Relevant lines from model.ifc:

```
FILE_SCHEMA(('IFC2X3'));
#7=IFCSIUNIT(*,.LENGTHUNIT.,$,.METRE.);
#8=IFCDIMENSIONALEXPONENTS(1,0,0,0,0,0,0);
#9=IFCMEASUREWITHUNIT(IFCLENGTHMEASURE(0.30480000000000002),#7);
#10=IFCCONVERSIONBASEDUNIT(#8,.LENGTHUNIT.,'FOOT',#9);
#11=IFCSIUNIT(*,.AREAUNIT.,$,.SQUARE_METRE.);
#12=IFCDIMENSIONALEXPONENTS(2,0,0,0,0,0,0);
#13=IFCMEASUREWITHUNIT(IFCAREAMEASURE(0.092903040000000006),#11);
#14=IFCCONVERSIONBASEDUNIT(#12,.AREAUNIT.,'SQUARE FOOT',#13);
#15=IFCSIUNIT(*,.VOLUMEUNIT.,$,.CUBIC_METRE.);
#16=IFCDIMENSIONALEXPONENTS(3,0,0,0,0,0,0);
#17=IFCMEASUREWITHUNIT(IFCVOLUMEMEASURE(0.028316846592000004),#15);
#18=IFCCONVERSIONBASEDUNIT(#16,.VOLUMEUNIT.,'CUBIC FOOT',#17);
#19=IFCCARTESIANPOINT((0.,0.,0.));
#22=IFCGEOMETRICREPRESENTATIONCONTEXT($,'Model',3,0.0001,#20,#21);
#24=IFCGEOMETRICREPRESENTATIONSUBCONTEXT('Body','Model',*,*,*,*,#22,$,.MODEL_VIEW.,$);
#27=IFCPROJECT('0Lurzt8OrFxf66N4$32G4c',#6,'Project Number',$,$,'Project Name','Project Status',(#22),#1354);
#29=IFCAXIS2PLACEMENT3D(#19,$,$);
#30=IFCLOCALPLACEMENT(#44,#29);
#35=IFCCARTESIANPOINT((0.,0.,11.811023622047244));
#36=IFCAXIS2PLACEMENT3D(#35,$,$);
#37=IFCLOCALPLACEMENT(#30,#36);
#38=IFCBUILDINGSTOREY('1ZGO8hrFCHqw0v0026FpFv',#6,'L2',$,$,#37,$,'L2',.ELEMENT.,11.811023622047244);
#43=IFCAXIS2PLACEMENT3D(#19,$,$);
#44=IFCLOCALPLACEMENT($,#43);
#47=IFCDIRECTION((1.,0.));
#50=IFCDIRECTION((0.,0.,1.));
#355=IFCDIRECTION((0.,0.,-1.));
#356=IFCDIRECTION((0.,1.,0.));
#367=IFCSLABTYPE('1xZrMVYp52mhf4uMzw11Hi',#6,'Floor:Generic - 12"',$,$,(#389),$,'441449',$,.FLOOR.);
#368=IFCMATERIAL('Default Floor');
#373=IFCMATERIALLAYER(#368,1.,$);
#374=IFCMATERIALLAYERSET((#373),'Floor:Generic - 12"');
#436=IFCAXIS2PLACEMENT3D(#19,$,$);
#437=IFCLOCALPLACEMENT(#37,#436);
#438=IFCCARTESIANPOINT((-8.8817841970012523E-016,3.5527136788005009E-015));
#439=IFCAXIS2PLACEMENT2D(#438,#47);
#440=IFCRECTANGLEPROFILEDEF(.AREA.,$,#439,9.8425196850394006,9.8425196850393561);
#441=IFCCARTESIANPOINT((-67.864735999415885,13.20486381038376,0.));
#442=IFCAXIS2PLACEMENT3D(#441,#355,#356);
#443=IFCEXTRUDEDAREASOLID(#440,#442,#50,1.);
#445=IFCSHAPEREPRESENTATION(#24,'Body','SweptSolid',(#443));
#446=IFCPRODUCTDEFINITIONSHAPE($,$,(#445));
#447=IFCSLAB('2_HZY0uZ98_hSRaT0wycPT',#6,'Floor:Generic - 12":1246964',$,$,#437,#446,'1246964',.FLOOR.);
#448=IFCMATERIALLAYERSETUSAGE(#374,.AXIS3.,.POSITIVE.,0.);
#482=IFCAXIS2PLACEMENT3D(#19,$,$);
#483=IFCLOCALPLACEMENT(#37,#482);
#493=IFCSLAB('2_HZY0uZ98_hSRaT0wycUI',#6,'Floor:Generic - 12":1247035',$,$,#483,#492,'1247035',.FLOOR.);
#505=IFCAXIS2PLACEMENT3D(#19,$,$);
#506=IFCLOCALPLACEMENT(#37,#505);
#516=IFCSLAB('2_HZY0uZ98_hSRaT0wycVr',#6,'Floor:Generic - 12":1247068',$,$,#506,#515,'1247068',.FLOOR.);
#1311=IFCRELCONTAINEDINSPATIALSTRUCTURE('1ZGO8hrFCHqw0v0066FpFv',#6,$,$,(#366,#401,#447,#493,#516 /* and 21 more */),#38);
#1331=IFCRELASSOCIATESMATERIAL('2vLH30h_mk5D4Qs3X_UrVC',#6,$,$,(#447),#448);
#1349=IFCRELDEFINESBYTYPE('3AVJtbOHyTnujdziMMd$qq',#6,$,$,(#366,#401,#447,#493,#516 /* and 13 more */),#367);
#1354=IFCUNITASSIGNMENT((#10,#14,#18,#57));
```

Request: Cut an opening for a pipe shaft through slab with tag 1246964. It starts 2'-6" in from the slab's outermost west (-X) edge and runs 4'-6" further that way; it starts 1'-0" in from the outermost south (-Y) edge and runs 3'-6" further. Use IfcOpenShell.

```python
import numpy as np
import ifcopenshell
import ifcopenshell.api.feature
import ifcopenshell.api.geometry
import ifcopenshell.api.root
import ifcopenshell.geom
import ifcopenshell.util.placement
import ifcopenshell.util.representation
import ifcopenshell.util.shape
import ifcopenshell.util.unit

model = ifcopenshell.open("model.ifc")
unit_scale = ifcopenshell.util.unit.calculate_unit_scale(model)
settings = ifcopenshell.geom.settings()


def volume(element):
    """Net volume in cubic metres, openings subtracted."""
    shape = ifcopenshell.geom.create_shape(settings, element)
    return ifcopenshell.util.shape.get_volume(shape.geometry)


slab = model.by_guid("2_HZY0uZ98_hSRaT0wycPT")
before = volume(slab)

# Extent in the slab's own axes, in metres. The edges named are its -X and -Y sides.
slab_shape = ifcopenshell.geom.create_shape(settings, slab)
vertices = ifcopenshell.util.shape.get_vertices(slab_shape.geometry)
x_min, y_min, bottom = vertices.min(axis=0)
top = vertices[:, 2].max()

opening = ifcopenshell.api.root.create_entity(model, ifc_class="IfcOpeningElement", name="Pipe shaft opening")
context = ifcopenshell.util.representation.get_context(model, "Model", "Body", "MODEL_VIEW")
width, depth = 1.3716, 1.0668
outline = [(0.0, 0.0), (width, 0.0), (width, depth), (0.0, depth), (0.0, 0.0)]
# Overshoot both faces by 50 mm so the cut is clean.
shape = ifcopenshell.api.geometry.add_slab_representation(
    model, context=context, depth=top - bottom + 0.1, polyline=outline
)
ifcopenshell.api.geometry.assign_representation(model, product=opening, representation=shape)

matrix = ifcopenshell.util.placement.get_local_placement(slab.ObjectPlacement)
matrix[:, 3] = matrix @ np.append(np.array([x_min + 0.762, y_min + 0.3048, bottom - 0.05]) / unit_scale, 1.0)
ifcopenshell.api.geometry.edit_object_placement(model, product=opening, matrix=matrix, is_si=False)
ifcopenshell.api.feature.add_feature(model, feature=opening, element=slab)

after = volume(slab)

print(f"slab volume {before:.3f} -> {after:.3f} m3")

model.write("model_updated.ifc")
```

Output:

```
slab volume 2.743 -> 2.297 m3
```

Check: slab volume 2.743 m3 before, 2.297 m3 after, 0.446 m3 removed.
